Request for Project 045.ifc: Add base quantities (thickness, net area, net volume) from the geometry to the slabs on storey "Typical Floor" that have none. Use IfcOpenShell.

First a look at what the model holds.

```python
import ifcopenshell
import ifcopenshell.util.element
import ifcopenshell.util.unit

model = ifcopenshell.open("Project 045.ifc")
print(model.schema)
for unit_type in ("LENGTHUNIT", "AREAUNIT", "VOLUMEUNIT"):
    print(unit_type, ifcopenshell.util.unit.calculate_unit_scale(model, unit_type))
storey = next(s for s in model.by_type("IfcBuildingStorey") if s.Name == "Typical Floor")
slabs = [e for e in ifcopenshell.util.element.get_decomposition(storey) if e.is_a("IfcSlab")]
for e in sorted(slabs, key=lambda e: e.id()):
    print(e.id(), e.is_a(), e.Name, list(ifcopenshell.util.element.get_psets(e, qtos_only=True)), sep=" | ")
```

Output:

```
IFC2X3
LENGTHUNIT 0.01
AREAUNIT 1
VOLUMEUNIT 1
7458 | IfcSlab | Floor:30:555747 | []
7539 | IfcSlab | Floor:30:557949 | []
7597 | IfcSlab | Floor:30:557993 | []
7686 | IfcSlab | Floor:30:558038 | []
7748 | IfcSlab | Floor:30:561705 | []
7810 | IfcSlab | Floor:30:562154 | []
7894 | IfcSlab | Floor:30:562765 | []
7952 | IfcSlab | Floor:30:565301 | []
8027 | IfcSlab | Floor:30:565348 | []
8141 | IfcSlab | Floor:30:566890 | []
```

```python
import ifcopenshell
import ifcopenshell.api.pset
import ifcopenshell.geom
import ifcopenshell.util.element
import ifcopenshell.util.shape
import ifcopenshell.util.unit

model = ifcopenshell.open("Project 045.ifc")
unit_scale = ifcopenshell.util.unit.calculate_unit_scale(model)
area_scale = ifcopenshell.util.unit.calculate_unit_scale(model, "AREAUNIT")
volume_scale = ifcopenshell.util.unit.calculate_unit_scale(model, "VOLUMEUNIT")
settings = ifcopenshell.geom.settings()

storey = next(s for s in model.by_type("IfcBuildingStorey") if s.Name == "Typical Floor")
slabs = [e for e in ifcopenshell.util.element.get_decomposition(storey) if e.is_a("IfcSlab")]

for e in sorted(slabs, key=lambda e: e.id()):
    if ifcopenshell.util.element.get_psets(e, qtos_only=True, should_inherit=False):
        continue
    # Geometry comes back in metres, in the element's own axes.
    shape = ifcopenshell.geom.create_shape(settings, e)
    values = {
        "Width": ifcopenshell.util.shape.get_z(shape.geometry) / unit_scale,
        "NetArea": ifcopenshell.util.shape.get_footprint_area(shape.geometry) / area_scale,
        "NetVolume": ifcopenshell.util.shape.get_volume(shape.geometry) / volume_scale,
    }
    qto = ifcopenshell.api.pset.add_qto(model, product=e, name="BaseQuantities")
    ifcopenshell.api.pset.edit_qto(model, qto=qto, properties=values)
    print(e.id(), {k: round(v, 3) for k, v in values.items()})

model.write("Project 045-out.ifc")
```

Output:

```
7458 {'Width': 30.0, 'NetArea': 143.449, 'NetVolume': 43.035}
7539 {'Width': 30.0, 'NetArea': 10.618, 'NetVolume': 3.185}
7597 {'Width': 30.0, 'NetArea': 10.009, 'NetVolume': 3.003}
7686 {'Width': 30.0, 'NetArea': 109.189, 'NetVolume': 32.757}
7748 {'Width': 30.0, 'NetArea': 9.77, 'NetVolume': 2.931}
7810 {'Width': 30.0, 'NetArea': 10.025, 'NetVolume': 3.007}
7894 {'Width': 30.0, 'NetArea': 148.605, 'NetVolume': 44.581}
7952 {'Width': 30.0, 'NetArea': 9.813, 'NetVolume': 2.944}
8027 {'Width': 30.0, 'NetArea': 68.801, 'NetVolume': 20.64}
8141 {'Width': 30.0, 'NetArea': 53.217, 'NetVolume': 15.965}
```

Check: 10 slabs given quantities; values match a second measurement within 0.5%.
